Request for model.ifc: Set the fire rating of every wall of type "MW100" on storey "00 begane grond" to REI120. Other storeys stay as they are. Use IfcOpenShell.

First a look at what the model holds.

```python
import ifcopenshell
import ifcopenshell.util.element

model = ifcopenshell.open("model.ifc")
print(model.schema)
storey = next(s for s in model.by_type("IfcBuildingStorey") if s.Name == "00 begane grond")
walls = [e for e in ifcopenshell.util.element.get_decomposition(storey) if e.is_a("IfcWall")]
seen = {}
for e in walls:
    element_type = ifcopenshell.util.element.get_type(e)
    key = (element_type.Name if element_type != e and element_type else None, ifcopenshell.util.element.get_pset(e, "Pset_WallCommon", "FireRating"))
    seen[key] = seen.get(key, 0) + 1
for (name, value), count in sorted(seen.items(), key=str):
    print(count, "x", name, "|", value)
```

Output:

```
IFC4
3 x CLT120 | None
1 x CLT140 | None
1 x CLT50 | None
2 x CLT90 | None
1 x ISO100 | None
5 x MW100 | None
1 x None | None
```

```python
import ifcopenshell
import ifcopenshell.api.pset
import ifcopenshell.util.element

model = ifcopenshell.open("model.ifc")

storey = next(s for s in model.by_type("IfcBuildingStorey") if s.Name == "00 begane grond")
walls = [e for e in ifcopenshell.util.element.get_decomposition(storey) if e.is_a("IfcWall")]

count = 0
for e in walls:
    element_type = ifcopenshell.util.element.get_type(e)
    if element_type in (None, e) or element_type.Name != "MW100":
        continue
    # add_pset returns the element's existing set when there is one.
    pset = ifcopenshell.api.pset.add_pset(model, product=e, name="Pset_WallCommon")
    ifcopenshell.api.pset.edit_pset(model, pset=pset, properties={"FireRating": "REI120"})
    count += 1

print(count, "walls updated")

model.write("model_rev.ifc")
```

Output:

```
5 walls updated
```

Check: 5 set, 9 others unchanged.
